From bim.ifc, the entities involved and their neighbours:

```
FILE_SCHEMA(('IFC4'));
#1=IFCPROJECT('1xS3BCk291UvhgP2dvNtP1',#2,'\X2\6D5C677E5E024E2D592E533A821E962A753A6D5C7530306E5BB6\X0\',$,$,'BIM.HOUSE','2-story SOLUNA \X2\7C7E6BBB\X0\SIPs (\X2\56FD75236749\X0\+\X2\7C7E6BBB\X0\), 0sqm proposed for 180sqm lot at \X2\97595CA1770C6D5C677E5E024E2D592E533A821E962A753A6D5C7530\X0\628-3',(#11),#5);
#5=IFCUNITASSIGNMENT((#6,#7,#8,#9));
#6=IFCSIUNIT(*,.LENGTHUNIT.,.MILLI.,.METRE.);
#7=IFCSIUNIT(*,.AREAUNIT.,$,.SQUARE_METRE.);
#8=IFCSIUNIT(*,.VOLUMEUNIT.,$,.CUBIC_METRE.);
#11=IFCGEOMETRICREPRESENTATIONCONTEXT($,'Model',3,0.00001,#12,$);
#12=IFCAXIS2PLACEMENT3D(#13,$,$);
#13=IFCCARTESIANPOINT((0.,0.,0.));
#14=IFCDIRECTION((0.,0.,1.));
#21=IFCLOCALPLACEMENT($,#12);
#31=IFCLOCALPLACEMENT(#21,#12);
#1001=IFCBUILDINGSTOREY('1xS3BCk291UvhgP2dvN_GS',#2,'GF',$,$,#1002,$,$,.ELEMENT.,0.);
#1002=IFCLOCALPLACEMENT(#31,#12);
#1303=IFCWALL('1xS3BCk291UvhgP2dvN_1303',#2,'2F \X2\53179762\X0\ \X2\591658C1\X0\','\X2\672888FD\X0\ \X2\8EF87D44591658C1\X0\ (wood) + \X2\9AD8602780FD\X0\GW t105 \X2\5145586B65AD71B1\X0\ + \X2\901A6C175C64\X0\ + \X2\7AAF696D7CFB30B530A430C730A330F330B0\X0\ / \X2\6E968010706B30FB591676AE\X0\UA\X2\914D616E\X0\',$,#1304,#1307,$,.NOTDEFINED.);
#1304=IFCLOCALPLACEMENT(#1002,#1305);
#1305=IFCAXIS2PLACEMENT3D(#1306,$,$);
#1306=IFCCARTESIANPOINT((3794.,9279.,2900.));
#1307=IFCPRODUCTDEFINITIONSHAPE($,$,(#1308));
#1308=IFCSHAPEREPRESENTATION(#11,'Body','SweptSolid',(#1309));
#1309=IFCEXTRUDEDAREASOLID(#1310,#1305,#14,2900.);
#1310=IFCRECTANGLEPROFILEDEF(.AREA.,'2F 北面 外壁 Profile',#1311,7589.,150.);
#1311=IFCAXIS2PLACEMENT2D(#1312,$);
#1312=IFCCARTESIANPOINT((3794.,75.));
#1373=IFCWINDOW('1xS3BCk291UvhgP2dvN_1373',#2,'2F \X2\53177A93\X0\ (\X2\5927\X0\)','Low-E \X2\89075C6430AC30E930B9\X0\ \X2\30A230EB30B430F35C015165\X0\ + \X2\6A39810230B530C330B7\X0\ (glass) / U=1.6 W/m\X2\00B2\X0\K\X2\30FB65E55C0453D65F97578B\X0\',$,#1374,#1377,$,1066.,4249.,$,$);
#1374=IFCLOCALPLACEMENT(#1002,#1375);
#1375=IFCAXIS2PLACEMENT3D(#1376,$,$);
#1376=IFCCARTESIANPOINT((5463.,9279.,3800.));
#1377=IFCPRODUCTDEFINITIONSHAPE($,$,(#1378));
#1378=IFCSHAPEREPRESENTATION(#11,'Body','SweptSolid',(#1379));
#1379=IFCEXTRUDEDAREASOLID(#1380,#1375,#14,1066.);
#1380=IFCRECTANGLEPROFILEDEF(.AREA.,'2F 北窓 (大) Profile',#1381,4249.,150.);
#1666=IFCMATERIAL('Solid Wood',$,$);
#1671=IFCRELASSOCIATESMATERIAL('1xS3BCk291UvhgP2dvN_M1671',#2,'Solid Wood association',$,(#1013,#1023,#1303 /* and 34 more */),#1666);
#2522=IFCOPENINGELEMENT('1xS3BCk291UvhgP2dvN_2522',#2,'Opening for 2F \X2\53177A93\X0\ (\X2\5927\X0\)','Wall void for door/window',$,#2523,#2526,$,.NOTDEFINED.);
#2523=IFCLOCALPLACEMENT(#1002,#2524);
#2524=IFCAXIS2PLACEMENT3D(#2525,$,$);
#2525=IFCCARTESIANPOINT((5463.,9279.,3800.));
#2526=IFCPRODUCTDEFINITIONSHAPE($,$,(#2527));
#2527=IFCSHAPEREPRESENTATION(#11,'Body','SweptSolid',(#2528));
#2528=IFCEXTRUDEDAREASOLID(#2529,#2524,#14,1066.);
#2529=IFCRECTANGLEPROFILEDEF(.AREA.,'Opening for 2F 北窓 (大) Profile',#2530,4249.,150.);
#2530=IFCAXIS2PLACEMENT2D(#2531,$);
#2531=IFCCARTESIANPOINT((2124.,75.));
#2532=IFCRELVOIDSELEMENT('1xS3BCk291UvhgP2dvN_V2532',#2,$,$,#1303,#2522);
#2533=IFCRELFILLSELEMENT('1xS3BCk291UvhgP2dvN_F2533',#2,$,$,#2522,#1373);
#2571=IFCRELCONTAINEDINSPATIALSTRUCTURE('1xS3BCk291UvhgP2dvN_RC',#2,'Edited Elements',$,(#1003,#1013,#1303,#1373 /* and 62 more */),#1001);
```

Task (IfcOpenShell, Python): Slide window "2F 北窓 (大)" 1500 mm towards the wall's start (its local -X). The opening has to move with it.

```python
import ifcopenshell
import ifcopenshell.api.geometry
import ifcopenshell.util.placement

model = ifcopenshell.open("bim.ifc")

window = model.by_guid("1xS3BCk291UvhgP2dvN_1373")
opening = window.FillsVoids[0].RelatingOpeningElement
wall = opening.VoidsElements[0].RelatingBuildingElement

wall_matrix = ifcopenshell.util.placement.get_local_placement(wall.ObjectPlacement)
shift = wall_matrix[:3, 0] * -1500.0
before = ifcopenshell.util.placement.get_local_placement(window.ObjectPlacement)[:3, 3].copy()

# The window is not placed relative to its opening, so move both.
for product in (opening, window):
    matrix = ifcopenshell.util.placement.get_local_placement(product.ObjectPlacement)
    matrix[:3, 3] += shift
    ifcopenshell.api.geometry.edit_object_placement(model, product=product, matrix=matrix, is_si=False)

after = ifcopenshell.util.placement.get_local_placement(window.ObjectPlacement)[:3, 3]
print("window moved by", (after - before).round(3) + 0.0)

model.write("bim_v2.ifc")
```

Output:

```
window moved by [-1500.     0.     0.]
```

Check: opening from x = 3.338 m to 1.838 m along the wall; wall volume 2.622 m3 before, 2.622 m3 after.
